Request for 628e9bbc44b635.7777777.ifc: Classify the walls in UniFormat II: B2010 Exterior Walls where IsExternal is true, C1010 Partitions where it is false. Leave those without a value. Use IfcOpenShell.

First a look at what the model holds.

```python
import ifcopenshell
import ifcopenshell.util.element

model = ifcopenshell.open("628e9bbc44b635.7777777.ifc")
print(model.schema)
print("classifications:", [c.Name for c in model.by_type("IfcClassification")])
values = [ifcopenshell.util.element.get_pset(e, "Pset_WallCommon", "IsExternal") for e in model.by_type("IfcWall")]
for value in (True, False, None):
    print("IsExternal", value, values.count(value))
```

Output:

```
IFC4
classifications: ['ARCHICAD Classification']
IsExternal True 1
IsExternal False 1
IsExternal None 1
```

```python
import ifcopenshell
import ifcopenshell.api.classification
import ifcopenshell.util.element

model = ifcopenshell.open("628e9bbc44b635.7777777.ifc")

system = ifcopenshell.api.classification.add_classification(model, classification="UniFormat II")

walls = model.by_type("IfcWall")
external = {e: ifcopenshell.util.element.get_pset(e, "Pset_WallCommon", "IsExternal") for e in walls}
for flag, code, name in ((True, "B2010", "Exterior Walls"), (False, "C1010", "Partitions")):
    products = [e for e in walls if external[e] is flag]
    ifcopenshell.api.classification.add_reference(
        model, products=products, classification=system, identification=code, name=name
    )
    print(code, len(products))

model.write("628e9bbc44b635.7777777-out.ifc")
```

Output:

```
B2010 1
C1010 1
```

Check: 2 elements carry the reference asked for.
